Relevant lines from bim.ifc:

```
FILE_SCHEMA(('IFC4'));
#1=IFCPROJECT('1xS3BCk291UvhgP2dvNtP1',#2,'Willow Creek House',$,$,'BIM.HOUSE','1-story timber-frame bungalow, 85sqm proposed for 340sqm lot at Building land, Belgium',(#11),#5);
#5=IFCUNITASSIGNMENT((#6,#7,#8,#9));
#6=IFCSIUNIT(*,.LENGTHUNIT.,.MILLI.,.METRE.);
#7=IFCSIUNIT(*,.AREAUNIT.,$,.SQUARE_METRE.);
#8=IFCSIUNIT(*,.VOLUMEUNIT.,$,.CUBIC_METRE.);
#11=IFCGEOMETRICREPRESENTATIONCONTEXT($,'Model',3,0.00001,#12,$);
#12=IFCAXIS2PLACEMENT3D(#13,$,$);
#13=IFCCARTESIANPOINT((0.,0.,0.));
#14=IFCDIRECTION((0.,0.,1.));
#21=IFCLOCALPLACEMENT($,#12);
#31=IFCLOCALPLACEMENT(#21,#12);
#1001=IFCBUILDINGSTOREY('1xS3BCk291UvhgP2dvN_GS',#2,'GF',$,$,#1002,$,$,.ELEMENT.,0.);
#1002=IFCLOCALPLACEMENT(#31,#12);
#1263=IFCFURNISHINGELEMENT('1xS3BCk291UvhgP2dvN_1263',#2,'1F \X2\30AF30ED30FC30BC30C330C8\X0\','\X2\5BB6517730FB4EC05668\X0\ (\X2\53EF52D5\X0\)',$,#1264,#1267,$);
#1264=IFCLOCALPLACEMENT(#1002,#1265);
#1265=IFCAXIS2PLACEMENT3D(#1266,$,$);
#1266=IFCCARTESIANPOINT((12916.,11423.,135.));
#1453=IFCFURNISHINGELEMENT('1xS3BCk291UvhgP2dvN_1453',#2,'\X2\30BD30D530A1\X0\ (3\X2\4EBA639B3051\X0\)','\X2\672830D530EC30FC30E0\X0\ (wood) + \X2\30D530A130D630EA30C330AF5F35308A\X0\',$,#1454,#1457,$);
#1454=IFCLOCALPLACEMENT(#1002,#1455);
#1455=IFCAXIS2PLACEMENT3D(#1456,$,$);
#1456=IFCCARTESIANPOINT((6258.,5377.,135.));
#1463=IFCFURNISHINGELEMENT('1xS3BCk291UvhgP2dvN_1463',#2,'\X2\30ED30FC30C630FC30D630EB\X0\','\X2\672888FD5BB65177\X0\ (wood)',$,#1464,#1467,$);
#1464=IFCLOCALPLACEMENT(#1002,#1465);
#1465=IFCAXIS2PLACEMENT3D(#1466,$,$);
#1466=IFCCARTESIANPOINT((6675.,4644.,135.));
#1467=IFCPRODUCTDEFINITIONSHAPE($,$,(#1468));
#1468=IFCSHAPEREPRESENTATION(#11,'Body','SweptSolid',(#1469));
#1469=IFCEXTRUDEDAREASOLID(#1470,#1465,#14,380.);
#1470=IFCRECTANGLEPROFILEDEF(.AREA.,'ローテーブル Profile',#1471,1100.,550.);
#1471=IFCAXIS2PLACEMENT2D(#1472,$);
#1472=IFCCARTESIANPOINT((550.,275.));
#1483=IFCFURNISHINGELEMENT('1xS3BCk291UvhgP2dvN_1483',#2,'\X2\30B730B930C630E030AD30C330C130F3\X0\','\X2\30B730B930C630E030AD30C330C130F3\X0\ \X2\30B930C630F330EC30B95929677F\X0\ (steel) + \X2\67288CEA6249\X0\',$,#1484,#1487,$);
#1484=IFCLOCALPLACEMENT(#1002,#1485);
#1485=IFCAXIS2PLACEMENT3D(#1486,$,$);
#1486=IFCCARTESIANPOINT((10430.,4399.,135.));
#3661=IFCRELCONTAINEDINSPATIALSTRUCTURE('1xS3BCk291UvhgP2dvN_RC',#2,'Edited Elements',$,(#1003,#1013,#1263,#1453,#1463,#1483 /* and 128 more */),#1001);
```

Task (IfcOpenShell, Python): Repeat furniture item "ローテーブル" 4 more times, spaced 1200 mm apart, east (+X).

```python
import numpy as np
import ifcopenshell
import ifcopenshell.api.geometry
import ifcopenshell.api.root
import ifcopenshell.util.element
import ifcopenshell.util.placement
import ifcopenshell.util.unit

model = ifcopenshell.open("bim.ifc")
unit_scale = ifcopenshell.util.unit.calculate_unit_scale(model)


def reuse_history(source, copy):
    """copy_class also copies each property set's owner history, people and application; keep the originals."""
    for rel in copy.IsDefinedBy:
        if rel.is_a("IfcRelDefinesByProperties") and (history := rel.RelatingPropertyDefinition.OwnerHistory):
            rel.RelatingPropertyDefinition.OwnerHistory = source.OwnerHistory
            ifcopenshell.util.element.remove_deep2(model, history)


source = model.by_guid("1xS3BCk291UvhgP2dvN_1463")
base = ifcopenshell.util.placement.get_local_placement(source.ObjectPlacement)
step = np.array([1.0, 0.0, 0.0]) * 1.2 / unit_scale

for i in range(1, 5):
    copy = ifcopenshell.api.root.copy_class(model, product=source)
    copy.Representation = ifcopenshell.util.element.copy_deep(
        model, source.Representation, exclude=["IfcGeometricRepresentationContext", "IfcRepresentationMap"]
    )
    reuse_history(source, copy)
    matrix = base.copy()
    matrix[:3, 3] += i * step
    print("added at", matrix[:3, 3].round(3) + 0.0)
    ifcopenshell.api.geometry.edit_object_placement(model, product=copy, matrix=matrix, is_si=False)

model.write("bim_rev.ifc")
```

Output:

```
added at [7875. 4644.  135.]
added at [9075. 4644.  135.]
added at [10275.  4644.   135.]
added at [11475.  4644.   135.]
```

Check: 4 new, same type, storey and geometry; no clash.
